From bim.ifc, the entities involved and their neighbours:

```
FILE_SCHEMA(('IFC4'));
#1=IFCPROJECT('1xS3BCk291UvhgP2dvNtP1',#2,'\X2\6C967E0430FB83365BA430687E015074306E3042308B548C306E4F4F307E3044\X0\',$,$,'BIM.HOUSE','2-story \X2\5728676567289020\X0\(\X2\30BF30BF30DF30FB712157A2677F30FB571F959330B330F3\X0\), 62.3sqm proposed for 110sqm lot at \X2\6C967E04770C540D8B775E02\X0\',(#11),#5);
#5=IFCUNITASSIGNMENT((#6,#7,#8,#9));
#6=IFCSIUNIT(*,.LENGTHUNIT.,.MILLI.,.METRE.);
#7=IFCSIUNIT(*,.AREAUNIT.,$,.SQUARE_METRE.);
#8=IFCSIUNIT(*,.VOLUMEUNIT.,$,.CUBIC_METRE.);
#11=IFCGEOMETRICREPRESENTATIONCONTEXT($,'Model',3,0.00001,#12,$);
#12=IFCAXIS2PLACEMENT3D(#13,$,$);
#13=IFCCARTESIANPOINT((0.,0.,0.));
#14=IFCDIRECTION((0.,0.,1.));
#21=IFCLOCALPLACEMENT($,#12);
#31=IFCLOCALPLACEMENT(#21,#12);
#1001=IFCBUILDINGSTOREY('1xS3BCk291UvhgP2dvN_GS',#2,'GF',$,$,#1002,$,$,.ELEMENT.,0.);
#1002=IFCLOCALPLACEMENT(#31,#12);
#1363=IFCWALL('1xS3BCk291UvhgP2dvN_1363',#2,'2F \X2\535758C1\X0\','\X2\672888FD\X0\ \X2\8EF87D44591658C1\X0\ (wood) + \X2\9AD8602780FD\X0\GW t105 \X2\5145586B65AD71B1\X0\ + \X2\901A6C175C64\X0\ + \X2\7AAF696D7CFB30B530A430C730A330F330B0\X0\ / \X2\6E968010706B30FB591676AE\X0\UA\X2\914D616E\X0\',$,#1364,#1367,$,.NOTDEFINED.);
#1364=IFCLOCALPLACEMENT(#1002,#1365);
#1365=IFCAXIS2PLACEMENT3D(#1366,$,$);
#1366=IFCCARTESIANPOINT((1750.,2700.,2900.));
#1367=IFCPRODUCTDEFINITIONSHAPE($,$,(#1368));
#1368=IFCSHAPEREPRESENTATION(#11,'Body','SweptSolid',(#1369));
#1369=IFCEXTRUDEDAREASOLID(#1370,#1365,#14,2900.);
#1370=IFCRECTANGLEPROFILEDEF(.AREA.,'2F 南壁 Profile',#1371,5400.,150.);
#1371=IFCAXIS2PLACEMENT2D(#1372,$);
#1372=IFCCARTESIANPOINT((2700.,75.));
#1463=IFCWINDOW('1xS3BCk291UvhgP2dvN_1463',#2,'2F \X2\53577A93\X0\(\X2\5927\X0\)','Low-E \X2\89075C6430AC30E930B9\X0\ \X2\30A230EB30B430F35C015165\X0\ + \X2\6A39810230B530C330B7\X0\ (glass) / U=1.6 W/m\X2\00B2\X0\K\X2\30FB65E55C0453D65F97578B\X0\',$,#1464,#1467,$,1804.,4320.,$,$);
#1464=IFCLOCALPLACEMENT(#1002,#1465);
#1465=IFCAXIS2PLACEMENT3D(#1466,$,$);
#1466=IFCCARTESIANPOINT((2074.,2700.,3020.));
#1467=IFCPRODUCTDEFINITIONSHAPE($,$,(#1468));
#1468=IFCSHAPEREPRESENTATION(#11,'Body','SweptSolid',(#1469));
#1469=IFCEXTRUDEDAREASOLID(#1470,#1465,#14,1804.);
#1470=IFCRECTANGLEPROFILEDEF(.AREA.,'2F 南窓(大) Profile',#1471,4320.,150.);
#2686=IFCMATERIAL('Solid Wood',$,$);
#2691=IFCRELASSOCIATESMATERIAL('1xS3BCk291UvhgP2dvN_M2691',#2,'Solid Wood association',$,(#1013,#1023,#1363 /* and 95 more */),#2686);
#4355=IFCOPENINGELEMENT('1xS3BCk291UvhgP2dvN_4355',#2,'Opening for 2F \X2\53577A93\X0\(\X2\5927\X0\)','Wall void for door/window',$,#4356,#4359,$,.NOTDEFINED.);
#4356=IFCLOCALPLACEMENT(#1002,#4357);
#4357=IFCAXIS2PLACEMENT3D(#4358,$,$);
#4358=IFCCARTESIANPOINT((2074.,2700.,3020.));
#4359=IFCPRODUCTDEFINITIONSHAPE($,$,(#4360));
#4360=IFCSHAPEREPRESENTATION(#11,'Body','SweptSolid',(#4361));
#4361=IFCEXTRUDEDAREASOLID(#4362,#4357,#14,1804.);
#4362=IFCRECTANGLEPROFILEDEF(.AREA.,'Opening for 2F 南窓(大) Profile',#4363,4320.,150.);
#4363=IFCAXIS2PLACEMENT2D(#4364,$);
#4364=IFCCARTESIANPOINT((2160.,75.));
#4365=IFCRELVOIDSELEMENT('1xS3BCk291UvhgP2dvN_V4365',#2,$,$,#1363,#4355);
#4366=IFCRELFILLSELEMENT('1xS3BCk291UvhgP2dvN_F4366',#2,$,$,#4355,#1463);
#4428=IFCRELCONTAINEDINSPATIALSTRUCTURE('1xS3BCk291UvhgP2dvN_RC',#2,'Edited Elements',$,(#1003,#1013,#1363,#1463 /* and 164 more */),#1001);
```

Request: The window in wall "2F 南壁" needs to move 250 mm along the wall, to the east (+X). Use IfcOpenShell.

```python
import ifcopenshell
import ifcopenshell.api.geometry
import ifcopenshell.util.placement
import ifcopenshell.util.unit

model = ifcopenshell.open("bim.ifc")
unit_scale = ifcopenshell.util.unit.calculate_unit_scale(model)

window = model.by_id(1463)
opening = window.FillsVoids[0].RelatingOpeningElement
wall = opening.VoidsElements[0].RelatingBuildingElement

wall_matrix = ifcopenshell.util.placement.get_local_placement(wall.ObjectPlacement)
shift = wall_matrix[:3, 0] * 0.25 / unit_scale
before = ifcopenshell.util.placement.get_local_placement(window.ObjectPlacement)[:3, 3].copy()

# The window is not placed relative to its opening, so move both.
for product in (opening, window):
    matrix = ifcopenshell.util.placement.get_local_placement(product.ObjectPlacement)
    matrix[:3, 3] += shift
    ifcopenshell.api.geometry.edit_object_placement(model, product=product, matrix=matrix, is_si=False)

after = ifcopenshell.util.placement.get_local_placement(window.ObjectPlacement)[:3, 3]
print("window moved by", (after - before).round(3) + 0.0)

model.write("bim_rev.ifc")
```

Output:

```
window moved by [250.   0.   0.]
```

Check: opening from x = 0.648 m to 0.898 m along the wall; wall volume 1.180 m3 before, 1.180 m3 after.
